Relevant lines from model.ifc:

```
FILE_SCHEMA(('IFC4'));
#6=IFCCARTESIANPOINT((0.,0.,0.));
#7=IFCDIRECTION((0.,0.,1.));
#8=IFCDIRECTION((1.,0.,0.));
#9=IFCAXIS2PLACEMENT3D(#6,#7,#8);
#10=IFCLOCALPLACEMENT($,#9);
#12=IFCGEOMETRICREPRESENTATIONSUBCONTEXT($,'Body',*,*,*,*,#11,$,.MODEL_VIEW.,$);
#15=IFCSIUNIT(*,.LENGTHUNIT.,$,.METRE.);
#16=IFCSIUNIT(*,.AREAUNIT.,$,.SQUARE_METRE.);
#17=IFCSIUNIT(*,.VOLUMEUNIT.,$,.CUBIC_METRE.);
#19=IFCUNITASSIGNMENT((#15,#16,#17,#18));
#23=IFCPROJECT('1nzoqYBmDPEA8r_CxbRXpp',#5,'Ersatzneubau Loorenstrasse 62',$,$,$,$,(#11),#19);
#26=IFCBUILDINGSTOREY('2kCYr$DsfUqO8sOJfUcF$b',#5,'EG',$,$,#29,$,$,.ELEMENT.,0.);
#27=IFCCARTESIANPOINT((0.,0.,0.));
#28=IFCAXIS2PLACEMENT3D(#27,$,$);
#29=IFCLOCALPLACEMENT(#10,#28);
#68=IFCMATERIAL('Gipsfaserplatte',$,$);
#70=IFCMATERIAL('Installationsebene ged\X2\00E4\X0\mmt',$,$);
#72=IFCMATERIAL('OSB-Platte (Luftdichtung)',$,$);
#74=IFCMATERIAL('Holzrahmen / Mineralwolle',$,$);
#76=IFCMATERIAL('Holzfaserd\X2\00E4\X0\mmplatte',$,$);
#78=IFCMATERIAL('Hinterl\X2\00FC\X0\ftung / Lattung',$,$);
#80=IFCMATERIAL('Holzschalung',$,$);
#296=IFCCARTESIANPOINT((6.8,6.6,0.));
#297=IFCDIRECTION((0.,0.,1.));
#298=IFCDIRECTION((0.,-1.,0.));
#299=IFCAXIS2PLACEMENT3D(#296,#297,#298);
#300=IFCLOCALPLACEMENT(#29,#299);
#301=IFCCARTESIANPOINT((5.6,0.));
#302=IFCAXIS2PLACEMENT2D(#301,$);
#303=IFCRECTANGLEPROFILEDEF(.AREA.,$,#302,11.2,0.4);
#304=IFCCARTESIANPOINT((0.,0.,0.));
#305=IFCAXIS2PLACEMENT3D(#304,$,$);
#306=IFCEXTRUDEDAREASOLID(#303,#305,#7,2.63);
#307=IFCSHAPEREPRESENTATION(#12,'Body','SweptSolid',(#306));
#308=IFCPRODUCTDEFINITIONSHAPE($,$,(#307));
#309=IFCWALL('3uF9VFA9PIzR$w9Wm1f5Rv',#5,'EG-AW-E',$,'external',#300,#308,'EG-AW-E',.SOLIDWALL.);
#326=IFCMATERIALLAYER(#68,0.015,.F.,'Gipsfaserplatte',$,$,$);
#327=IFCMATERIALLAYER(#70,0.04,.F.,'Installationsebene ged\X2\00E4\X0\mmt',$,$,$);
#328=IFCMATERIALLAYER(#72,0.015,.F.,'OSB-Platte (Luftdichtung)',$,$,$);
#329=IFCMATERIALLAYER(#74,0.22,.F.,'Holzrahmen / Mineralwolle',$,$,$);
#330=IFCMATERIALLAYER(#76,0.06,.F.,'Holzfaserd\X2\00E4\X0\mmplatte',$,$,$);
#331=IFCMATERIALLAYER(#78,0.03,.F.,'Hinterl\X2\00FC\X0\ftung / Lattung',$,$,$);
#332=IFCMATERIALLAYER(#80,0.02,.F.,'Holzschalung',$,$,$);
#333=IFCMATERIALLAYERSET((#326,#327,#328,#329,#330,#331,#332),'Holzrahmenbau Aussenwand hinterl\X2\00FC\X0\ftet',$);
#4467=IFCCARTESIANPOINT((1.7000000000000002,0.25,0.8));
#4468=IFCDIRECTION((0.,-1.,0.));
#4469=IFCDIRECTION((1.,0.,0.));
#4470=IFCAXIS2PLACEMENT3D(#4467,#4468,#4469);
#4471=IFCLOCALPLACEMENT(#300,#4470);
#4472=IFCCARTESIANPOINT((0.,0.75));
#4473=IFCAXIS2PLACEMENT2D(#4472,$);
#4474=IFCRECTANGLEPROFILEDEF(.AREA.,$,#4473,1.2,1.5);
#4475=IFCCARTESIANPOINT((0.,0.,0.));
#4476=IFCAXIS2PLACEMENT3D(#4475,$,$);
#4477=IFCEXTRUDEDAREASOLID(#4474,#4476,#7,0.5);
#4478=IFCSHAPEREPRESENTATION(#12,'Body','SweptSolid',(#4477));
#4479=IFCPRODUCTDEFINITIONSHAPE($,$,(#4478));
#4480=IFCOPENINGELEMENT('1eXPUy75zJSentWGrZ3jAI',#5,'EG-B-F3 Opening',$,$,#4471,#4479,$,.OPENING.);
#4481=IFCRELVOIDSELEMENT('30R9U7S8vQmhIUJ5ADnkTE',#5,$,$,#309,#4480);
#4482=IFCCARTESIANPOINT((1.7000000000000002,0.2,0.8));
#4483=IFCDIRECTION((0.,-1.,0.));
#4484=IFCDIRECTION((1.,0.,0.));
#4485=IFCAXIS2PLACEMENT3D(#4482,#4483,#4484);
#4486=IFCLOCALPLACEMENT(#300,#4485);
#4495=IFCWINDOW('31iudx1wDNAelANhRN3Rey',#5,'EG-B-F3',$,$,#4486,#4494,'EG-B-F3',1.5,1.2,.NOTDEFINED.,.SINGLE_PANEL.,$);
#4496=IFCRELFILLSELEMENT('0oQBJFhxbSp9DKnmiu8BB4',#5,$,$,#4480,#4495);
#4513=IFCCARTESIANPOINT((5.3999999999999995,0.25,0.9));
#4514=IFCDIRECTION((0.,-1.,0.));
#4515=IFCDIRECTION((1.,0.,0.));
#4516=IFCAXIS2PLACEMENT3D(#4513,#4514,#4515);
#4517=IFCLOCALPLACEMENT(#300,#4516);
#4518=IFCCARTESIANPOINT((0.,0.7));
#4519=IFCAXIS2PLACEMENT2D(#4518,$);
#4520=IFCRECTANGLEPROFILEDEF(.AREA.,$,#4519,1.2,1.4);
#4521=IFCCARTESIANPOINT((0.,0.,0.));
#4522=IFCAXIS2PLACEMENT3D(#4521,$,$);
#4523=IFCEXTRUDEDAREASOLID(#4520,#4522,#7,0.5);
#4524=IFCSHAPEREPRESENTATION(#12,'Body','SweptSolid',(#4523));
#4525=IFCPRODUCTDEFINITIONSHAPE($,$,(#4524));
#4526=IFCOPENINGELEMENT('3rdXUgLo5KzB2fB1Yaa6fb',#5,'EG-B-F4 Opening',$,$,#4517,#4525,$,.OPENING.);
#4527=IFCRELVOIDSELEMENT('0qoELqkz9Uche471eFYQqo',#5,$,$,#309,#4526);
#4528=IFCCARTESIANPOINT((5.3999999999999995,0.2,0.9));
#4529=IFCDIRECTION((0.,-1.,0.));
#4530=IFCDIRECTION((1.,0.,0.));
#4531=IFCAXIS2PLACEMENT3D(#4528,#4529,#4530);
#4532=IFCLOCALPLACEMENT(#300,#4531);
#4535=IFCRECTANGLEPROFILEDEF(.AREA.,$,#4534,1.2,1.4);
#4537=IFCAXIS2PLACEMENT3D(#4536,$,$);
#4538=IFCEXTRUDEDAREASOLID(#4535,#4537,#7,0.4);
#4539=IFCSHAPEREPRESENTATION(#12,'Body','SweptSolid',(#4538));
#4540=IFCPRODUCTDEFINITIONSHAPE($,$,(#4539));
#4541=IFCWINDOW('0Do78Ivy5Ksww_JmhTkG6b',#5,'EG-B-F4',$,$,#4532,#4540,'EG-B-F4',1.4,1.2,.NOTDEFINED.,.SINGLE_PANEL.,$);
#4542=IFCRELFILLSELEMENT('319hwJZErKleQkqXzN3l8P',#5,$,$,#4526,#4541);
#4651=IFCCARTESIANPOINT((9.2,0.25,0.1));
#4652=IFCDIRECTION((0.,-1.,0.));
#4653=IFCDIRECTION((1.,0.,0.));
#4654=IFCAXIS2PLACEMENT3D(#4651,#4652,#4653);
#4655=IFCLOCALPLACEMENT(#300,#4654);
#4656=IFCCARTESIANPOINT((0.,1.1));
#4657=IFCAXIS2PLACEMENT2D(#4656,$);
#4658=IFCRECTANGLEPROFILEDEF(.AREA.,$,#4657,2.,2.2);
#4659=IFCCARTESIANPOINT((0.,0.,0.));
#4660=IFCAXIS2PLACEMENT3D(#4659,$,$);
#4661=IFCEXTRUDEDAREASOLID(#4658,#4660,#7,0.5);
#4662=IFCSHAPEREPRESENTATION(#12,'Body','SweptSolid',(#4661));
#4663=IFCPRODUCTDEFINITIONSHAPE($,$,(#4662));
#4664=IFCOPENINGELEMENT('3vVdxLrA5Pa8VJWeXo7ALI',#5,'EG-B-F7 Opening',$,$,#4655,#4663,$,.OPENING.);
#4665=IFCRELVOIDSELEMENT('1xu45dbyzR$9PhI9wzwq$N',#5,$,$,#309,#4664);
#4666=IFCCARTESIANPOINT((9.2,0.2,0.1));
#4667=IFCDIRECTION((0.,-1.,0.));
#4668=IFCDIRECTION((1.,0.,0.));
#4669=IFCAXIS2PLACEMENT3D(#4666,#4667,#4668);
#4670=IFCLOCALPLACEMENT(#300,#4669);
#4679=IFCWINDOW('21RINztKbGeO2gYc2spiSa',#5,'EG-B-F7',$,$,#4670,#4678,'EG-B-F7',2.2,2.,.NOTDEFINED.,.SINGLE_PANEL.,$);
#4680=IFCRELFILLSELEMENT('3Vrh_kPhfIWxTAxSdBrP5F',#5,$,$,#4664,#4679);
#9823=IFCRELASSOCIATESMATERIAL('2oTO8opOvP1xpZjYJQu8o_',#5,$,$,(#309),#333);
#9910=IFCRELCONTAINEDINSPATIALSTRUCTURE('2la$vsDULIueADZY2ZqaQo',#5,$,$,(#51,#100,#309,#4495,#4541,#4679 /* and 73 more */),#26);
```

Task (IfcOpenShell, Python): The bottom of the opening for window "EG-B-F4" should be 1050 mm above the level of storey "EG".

```python
import numpy as np
import ifcopenshell
import ifcopenshell.api.geometry
import ifcopenshell.geom
import ifcopenshell.util.element
import ifcopenshell.util.placement
import ifcopenshell.util.shape
import ifcopenshell.util.unit

model = ifcopenshell.open("model.ifc")
unit_scale = ifcopenshell.util.unit.calculate_unit_scale(model)

window = model.by_id(4541)
opening = window.FillsVoids[0].RelatingOpeningElement
storey = ifcopenshell.util.element.get_container(window, ifc_class="IfcBuildingStorey")
level = ifcopenshell.util.placement.get_local_placement(storey.ObjectPlacement)[2, 3]

# The opening's origin need not be at the sill, so measure its lowest point.
shape = ifcopenshell.geom.create_shape(ifcopenshell.geom.settings(), opening)
bottom = ifcopenshell.util.shape.get_shape_bottom_elevation(shape, shape.geometry) / unit_scale
dz = level + 1.05 / unit_scale - bottom

shift = np.array([0.0, 0.0, dz])
# The window is not placed relative to its opening, so move both.
for product in (opening, window):
    matrix = ifcopenshell.util.placement.get_local_placement(product.ObjectPlacement)
    matrix[:3, 3] += shift
    ifcopenshell.api.geometry.edit_object_placement(model, product=product, matrix=matrix, is_si=False)

print(f"moved by {dz * unit_scale:+.3f} m")

model.write("model-out.ifc")
```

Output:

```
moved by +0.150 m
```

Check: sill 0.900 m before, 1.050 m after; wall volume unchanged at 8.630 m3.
